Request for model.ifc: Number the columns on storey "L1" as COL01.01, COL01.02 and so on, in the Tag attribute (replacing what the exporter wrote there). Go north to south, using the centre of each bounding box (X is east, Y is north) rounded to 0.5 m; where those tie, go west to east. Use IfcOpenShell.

First a look at what the model holds.

```python
import ifcopenshell
import ifcopenshell.util.element
import ifcopenshell.util.placement

model = ifcopenshell.open("model.ifc")
print(model.schema)
storey = next(s for s in model.by_type("IfcBuildingStorey") if s.Name == "L1")
columns = [e for e in ifcopenshell.util.element.get_decomposition(storey) if e.is_a("IfcColumn")]
for e in sorted(columns, key=lambda e: e.id()):
    origin = ifcopenshell.util.placement.get_local_placement(e.ObjectPlacement)[:3, 3]
    print(e.id(), e.Tag, e.Name, origin.round(2) + 0.0, sep=" | ")
```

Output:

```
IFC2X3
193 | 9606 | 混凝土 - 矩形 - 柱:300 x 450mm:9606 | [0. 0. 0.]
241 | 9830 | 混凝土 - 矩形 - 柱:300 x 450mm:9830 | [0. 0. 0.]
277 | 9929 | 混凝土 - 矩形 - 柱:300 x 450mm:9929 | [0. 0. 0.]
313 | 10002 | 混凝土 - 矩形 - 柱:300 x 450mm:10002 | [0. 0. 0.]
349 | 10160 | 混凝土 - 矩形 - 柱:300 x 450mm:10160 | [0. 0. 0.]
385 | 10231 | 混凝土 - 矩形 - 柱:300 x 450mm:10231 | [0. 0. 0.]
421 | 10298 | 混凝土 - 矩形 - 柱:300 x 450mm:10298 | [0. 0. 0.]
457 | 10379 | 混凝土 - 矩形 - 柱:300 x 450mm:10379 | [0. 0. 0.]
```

```python
import ifcopenshell
import ifcopenshell.geom
import ifcopenshell.util.element
import ifcopenshell.util.shape

model = ifcopenshell.open("model.ifc")
settings = ifcopenshell.geom.settings()
settings.set("use-world-coords", True)


def centre(element):
    shape = ifcopenshell.geom.create_shape(settings, element)
    return ifcopenshell.util.shape.get_bbox_centroid(shape.geometry)


storey = next(s for s in model.by_type("IfcBuildingStorey") if s.Name == "L1")
columns = [e for e in ifcopenshell.util.element.get_decomposition(storey) if e.is_a("IfcColumn")]

# Insertion points can sit at a corner or the storey origin, so sort by the geometry (in metres).
centres = {e: centre(e) for e in columns}
columns.sort(key=lambda e: (-round(centres[e][1] / 0.5), centres[e][0]))

for i, e in enumerate(columns, start=1):
    number = f"COL01.{i:02d}"
    e.Tag = number
    print(e.id(), number)

model.write("model_rev.ifc")
```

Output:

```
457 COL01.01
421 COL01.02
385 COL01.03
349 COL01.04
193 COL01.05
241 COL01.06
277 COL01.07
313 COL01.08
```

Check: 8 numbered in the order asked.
